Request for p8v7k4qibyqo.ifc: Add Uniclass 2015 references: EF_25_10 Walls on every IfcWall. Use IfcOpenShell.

First a look at what the model holds.

```python
import ifcopenshell

model = ifcopenshell.open("p8v7k4qibyqo.ifc")
print(model.schema)
print("classifications:", [c.Name for c in model.by_type("IfcClassification")])
for ifc_class in ("IfcDoor", "IfcRoof", "IfcStair", "IfcWall", "IfcWindow"):
    print(ifc_class, len(model.by_type(ifc_class)))
```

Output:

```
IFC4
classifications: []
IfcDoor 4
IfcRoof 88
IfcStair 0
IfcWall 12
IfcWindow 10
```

```python
import ifcopenshell
import ifcopenshell.api.classification

model = ifcopenshell.open("p8v7k4qibyqo.ifc")

system = ifcopenshell.api.classification.add_classification(model, classification="Uniclass 2015")

codes = {
    "IfcWall": ("EF_25_10", "Walls"),
}
for ifc_class, (code, name) in codes.items():
    products = model.by_type(ifc_class)
    ifcopenshell.api.classification.add_reference(
        model, products=products, classification=system, identification=code, name=name
    )
    print(code, len(products))

model.write("p8v7k4qibyqo_v2.ifc")
```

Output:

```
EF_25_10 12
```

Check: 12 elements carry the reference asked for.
